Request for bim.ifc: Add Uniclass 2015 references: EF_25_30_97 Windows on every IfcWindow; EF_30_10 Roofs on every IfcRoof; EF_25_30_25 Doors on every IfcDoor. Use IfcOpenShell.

First a look at what the model holds.

```python
import ifcopenshell

model = ifcopenshell.open("bim.ifc")
print(model.schema)
print("classifications:", [c.Name for c in model.by_type("IfcClassification")])
for ifc_class in ("IfcDoor", "IfcRoof", "IfcStair", "IfcWall", "IfcWindow"):
    print(ifc_class, len(model.by_type(ifc_class)))
```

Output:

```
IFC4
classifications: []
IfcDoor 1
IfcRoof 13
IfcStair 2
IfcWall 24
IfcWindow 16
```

```python
import ifcopenshell
import ifcopenshell.api.classification

model = ifcopenshell.open("bim.ifc")

system = ifcopenshell.api.classification.add_classification(model, classification="Uniclass 2015")

codes = {
    "IfcWindow": ("EF_25_30_97", "Windows"),
    "IfcRoof": ("EF_30_10", "Roofs"),
    "IfcDoor": ("EF_25_30_25", "Doors"),
}
for ifc_class, (code, name) in codes.items():
    products = model.by_type(ifc_class)
    ifcopenshell.api.classification.add_reference(
        model, products=products, classification=system, identification=code, name=name
    )
    print(code, len(products))

model.write("bim-out.ifc")
```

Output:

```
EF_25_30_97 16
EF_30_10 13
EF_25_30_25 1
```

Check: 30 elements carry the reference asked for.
